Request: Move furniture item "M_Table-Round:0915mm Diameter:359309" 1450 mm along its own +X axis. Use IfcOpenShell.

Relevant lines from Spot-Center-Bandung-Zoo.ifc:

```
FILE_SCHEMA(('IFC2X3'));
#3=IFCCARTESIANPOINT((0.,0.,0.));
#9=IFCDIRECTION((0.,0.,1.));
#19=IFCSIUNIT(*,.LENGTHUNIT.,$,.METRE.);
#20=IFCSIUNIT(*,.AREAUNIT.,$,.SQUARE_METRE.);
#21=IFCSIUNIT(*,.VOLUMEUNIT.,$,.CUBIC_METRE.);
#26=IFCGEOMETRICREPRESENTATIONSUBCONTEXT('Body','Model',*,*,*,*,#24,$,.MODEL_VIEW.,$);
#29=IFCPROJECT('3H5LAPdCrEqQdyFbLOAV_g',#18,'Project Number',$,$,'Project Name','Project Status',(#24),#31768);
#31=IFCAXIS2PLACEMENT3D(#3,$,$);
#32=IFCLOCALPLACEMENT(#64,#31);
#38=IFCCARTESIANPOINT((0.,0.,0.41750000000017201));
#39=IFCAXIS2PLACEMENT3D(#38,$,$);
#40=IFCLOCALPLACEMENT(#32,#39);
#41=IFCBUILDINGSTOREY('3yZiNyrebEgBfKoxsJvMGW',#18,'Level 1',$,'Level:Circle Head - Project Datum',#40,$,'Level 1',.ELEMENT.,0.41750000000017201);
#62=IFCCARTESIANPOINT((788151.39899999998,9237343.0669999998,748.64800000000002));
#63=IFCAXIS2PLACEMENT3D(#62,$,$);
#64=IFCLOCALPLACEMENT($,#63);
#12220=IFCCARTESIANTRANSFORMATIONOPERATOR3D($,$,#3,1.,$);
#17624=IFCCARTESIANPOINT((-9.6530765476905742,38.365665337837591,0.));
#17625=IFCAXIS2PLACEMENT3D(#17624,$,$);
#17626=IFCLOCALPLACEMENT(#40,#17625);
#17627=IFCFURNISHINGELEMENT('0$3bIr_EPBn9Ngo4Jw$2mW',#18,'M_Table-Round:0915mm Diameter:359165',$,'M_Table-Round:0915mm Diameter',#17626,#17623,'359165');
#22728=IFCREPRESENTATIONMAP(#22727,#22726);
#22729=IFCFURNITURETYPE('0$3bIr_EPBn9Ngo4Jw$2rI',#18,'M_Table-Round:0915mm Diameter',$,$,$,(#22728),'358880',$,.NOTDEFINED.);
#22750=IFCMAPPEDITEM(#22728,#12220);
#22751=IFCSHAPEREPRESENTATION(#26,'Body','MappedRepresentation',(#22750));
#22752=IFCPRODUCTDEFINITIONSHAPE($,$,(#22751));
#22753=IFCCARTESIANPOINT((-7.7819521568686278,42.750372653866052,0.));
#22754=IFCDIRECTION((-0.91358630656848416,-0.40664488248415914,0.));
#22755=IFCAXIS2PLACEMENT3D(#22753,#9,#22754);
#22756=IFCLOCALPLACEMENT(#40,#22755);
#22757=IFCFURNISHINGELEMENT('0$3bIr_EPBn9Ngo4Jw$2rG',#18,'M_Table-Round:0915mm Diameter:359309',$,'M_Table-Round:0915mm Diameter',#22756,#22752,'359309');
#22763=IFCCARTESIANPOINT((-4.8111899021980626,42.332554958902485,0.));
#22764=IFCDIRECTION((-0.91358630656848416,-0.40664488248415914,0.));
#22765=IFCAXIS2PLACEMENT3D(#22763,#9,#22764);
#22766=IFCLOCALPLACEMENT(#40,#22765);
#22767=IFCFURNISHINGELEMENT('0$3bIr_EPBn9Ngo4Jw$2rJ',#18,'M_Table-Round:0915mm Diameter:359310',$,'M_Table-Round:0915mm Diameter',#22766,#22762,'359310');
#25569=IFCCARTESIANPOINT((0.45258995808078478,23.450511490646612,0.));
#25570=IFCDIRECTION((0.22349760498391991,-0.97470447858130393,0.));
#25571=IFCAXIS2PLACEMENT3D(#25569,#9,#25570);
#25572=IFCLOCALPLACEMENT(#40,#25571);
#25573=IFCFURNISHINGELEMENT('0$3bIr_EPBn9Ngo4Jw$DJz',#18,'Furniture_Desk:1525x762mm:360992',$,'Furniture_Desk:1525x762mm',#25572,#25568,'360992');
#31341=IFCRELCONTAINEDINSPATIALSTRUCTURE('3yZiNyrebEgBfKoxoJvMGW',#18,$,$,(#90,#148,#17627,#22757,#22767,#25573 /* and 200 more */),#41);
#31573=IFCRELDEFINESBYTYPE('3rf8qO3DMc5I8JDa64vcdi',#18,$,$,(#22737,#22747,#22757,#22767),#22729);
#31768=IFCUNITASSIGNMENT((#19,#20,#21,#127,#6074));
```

```python
import ifcopenshell
import ifcopenshell.api.geometry
import ifcopenshell.util.placement

model = ifcopenshell.open("Spot-Center-Bandung-Zoo.ifc")

item = model.by_guid("0$3bIr_EPBn9Ngo4Jw$2rG")
matrix = ifcopenshell.util.placement.get_local_placement(item.ObjectPlacement)
matrix[:3, 3] += matrix[:3, 0] * 1.45
ifcopenshell.api.geometry.edit_object_placement(model, product=item, matrix=matrix, is_si=False)

print(ifcopenshell.util.placement.get_local_placement(item.ObjectPlacement).round(3) + 0.0)

model.write("Spot-Center-Bandung-Zoo_edited.ifc")
```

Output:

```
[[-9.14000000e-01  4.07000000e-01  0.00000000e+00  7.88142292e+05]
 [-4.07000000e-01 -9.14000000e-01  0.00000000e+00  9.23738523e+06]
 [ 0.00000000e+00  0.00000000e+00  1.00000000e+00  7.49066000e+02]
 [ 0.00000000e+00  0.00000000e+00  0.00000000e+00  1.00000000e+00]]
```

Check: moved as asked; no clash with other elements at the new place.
